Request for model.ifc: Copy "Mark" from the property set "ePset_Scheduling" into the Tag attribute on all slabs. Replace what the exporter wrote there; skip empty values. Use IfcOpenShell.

First a look at what the model holds.

```python
import ifcopenshell
import ifcopenshell.util.element

model = ifcopenshell.open("model.ifc")
print(model.schema)
slabs = model.by_type("IfcSlab")
print(len(slabs), "slabs")
for e in slabs[:8]:
    source = ifcopenshell.util.element.get_pset(e, "ePset_Scheduling", "Mark")
    target = e.Tag
    print(e.id(), repr(source), repr(target), sep=" | ")
```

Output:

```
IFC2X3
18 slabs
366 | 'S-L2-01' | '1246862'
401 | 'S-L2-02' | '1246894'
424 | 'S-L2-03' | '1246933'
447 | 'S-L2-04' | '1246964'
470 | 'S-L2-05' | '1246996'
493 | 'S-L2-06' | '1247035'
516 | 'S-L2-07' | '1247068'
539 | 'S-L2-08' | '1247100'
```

```python
import ifcopenshell
import ifcopenshell.util.element

model = ifcopenshell.open("model.ifc")

count = 0
for e in model.by_type("IfcSlab"):
    value = ifcopenshell.util.element.get_pset(e, "ePset_Scheduling", "Mark")
    current = e.Tag
    if not value or not value.strip() or current == value:
        continue
    e.Tag = value
    count += 1

print(count, "slabs updated")

model.write("model_updated.ifc")
```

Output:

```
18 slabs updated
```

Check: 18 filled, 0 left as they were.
